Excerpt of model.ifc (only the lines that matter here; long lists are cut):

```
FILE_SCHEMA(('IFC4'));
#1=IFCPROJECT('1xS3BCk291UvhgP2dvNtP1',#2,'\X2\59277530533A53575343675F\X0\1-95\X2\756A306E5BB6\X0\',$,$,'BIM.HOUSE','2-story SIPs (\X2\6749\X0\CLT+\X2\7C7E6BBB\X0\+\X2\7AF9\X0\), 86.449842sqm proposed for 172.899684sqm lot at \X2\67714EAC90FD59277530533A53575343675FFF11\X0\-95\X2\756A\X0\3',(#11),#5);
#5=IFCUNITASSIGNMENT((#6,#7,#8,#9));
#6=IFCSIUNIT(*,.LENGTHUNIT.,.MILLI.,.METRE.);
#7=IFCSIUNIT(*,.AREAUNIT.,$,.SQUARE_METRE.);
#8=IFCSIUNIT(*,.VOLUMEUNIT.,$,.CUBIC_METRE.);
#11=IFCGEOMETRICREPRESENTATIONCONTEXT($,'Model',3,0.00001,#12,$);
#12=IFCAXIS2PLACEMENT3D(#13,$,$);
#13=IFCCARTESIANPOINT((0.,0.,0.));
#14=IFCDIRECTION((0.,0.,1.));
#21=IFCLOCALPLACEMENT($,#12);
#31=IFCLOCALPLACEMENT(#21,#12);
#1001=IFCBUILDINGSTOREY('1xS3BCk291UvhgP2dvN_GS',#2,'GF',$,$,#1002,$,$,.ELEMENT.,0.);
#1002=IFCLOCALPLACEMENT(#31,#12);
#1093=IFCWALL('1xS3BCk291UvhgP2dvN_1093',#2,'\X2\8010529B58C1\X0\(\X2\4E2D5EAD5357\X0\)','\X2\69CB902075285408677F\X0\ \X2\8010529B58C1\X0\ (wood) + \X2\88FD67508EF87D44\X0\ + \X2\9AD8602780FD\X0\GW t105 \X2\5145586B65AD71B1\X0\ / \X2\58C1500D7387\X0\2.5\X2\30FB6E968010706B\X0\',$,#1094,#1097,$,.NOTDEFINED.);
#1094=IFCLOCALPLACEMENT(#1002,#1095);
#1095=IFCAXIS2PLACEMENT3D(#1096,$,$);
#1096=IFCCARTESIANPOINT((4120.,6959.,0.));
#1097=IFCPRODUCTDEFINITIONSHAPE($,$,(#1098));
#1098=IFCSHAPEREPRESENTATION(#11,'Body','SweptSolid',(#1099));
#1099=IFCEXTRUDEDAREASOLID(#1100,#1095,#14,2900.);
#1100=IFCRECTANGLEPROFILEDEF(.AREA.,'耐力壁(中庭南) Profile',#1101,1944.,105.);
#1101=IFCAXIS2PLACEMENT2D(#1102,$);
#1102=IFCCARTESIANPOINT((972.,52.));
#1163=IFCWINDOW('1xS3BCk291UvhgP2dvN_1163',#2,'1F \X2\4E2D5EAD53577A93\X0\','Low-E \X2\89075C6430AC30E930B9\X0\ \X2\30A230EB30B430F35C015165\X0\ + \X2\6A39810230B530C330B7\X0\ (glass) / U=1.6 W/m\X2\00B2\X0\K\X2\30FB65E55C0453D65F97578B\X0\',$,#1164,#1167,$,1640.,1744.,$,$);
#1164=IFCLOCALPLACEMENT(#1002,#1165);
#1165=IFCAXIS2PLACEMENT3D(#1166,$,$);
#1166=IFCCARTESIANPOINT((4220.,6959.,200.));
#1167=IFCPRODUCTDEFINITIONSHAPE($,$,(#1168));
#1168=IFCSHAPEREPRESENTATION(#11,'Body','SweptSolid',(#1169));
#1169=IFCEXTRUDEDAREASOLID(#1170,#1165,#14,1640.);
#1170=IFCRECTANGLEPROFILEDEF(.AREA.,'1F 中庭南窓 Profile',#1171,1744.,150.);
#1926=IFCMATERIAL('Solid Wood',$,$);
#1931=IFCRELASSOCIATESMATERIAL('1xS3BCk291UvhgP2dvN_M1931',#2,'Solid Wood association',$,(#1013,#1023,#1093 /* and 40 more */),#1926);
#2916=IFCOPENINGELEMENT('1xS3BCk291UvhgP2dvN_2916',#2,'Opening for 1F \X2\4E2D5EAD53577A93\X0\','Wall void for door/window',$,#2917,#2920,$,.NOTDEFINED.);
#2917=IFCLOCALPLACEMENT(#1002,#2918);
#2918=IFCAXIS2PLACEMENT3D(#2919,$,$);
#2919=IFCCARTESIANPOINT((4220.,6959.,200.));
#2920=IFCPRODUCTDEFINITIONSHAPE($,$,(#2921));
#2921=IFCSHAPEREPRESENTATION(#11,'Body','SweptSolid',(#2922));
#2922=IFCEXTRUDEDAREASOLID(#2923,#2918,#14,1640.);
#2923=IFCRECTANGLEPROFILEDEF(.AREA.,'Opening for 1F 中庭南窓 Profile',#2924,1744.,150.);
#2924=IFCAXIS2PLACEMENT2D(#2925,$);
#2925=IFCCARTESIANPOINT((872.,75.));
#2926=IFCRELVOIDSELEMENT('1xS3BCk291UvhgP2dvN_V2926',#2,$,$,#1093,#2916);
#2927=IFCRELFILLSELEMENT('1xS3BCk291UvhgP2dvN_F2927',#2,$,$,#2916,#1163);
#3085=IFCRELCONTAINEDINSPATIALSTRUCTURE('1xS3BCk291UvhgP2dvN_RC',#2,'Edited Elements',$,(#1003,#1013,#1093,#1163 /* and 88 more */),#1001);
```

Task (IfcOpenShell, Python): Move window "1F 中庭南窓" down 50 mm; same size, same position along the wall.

```python
import numpy as np
import ifcopenshell
import ifcopenshell.api.geometry
import ifcopenshell.util.placement
import ifcopenshell.util.unit

model = ifcopenshell.open("model.ifc")
unit_scale = ifcopenshell.util.unit.calculate_unit_scale(model)

window = model.by_guid("1xS3BCk291UvhgP2dvN_1163")
opening = window.FillsVoids[0].RelatingOpeningElement
dz = -0.05 / unit_scale

shift = np.array([0.0, 0.0, dz])
# The window is not placed relative to its opening, so move both.
for product in (opening, window):
    matrix = ifcopenshell.util.placement.get_local_placement(product.ObjectPlacement)
    matrix[:3, 3] += shift
    ifcopenshell.api.geometry.edit_object_placement(model, product=product, matrix=matrix, is_si=False)

print(f"moved by {dz * unit_scale:+.3f} m")

model.write("model-out.ifc")
```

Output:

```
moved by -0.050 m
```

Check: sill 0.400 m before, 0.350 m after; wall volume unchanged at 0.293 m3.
